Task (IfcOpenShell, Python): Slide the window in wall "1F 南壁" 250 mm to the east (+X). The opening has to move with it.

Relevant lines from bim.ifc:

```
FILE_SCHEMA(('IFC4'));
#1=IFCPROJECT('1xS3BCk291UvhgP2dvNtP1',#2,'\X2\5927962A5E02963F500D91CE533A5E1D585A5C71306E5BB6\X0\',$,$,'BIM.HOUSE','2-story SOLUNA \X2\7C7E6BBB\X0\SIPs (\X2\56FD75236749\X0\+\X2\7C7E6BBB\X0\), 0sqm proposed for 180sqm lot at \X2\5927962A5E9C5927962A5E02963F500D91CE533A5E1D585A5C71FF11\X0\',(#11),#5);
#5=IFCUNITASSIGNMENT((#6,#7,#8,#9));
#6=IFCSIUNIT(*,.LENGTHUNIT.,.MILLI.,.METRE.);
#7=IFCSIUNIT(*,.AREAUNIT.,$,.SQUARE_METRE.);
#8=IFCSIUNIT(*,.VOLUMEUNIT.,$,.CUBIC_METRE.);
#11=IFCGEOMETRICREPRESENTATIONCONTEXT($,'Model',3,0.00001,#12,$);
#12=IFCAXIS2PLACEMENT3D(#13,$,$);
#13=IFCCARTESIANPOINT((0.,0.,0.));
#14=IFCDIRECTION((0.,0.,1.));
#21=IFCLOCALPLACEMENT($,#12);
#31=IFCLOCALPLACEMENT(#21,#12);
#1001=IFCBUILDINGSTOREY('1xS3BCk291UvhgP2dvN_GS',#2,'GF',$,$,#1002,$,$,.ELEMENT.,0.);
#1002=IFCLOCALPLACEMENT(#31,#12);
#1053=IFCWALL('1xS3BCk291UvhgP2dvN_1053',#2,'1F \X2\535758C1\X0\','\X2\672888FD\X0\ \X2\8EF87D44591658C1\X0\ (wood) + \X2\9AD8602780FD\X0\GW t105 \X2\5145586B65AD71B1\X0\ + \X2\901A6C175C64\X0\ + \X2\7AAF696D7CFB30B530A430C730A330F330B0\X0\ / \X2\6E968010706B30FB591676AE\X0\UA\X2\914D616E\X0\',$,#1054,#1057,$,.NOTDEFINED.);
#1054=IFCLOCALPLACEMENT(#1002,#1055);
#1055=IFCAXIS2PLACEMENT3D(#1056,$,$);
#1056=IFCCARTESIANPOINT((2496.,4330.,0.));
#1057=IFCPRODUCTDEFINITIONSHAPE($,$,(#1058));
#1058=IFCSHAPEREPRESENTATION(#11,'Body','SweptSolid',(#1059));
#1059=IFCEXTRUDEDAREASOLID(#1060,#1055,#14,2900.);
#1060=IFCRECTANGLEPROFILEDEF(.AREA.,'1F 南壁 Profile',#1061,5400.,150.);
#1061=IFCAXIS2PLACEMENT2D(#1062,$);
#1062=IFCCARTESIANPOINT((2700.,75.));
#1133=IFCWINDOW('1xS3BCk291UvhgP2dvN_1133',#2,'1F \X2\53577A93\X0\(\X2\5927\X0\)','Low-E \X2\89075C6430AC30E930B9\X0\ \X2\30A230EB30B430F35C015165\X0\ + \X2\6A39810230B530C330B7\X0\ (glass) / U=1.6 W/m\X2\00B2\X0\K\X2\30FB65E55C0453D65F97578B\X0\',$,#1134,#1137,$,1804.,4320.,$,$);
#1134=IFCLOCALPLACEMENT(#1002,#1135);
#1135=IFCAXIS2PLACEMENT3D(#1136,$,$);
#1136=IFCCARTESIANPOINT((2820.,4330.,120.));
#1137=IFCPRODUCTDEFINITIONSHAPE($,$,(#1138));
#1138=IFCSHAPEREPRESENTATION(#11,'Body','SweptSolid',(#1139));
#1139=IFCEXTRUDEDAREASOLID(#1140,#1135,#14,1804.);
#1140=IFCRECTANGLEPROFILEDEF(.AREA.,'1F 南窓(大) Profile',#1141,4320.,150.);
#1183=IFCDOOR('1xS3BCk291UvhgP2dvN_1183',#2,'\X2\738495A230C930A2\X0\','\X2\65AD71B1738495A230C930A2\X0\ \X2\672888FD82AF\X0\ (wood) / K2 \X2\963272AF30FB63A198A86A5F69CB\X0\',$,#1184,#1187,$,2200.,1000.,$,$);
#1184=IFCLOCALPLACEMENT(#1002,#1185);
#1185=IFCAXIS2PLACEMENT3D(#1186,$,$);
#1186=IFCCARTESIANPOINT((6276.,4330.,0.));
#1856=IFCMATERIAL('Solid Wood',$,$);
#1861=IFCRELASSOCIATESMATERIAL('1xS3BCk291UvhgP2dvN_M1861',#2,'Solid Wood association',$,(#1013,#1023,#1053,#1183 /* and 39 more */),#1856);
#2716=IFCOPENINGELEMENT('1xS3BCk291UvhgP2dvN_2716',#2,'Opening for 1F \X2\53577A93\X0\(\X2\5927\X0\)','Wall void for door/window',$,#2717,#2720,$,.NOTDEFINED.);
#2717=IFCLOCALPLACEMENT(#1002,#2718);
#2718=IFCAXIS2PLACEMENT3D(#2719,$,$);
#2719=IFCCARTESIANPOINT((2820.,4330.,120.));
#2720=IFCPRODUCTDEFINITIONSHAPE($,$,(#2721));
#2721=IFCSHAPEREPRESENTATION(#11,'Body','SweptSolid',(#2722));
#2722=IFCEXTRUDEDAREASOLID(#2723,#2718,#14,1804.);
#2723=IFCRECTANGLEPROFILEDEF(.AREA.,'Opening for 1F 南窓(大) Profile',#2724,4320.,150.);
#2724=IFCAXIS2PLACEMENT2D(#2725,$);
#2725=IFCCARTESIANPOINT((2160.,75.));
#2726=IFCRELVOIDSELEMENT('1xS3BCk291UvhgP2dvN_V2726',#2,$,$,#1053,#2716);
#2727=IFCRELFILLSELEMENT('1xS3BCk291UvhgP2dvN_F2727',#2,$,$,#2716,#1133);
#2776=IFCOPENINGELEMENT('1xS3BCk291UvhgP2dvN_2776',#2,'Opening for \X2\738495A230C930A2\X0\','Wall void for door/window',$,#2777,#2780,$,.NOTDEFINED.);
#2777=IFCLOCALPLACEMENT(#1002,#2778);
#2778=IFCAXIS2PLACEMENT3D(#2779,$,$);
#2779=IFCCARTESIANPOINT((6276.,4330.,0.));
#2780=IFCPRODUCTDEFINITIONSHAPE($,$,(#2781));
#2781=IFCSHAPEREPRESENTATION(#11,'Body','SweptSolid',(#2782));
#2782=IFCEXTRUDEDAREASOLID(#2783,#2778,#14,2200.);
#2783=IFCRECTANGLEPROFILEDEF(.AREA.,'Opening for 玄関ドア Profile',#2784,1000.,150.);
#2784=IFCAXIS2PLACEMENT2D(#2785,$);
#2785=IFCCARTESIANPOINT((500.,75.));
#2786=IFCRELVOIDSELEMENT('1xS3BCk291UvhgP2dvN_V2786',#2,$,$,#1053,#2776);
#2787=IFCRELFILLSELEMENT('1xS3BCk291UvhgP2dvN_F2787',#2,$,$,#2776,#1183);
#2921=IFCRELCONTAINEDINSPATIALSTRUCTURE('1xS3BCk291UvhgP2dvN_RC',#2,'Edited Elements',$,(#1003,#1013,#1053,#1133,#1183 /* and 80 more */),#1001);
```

```python
import ifcopenshell
import ifcopenshell.api.geometry
import ifcopenshell.util.placement
import ifcopenshell.util.unit

model = ifcopenshell.open("bim.ifc")
unit_scale = ifcopenshell.util.unit.calculate_unit_scale(model)

window = model.by_guid("1xS3BCk291UvhgP2dvN_1133")
opening = window.FillsVoids[0].RelatingOpeningElement
wall = opening.VoidsElements[0].RelatingBuildingElement

wall_matrix = ifcopenshell.util.placement.get_local_placement(wall.ObjectPlacement)
shift = wall_matrix[:3, 0] * 0.25 / unit_scale
before = ifcopenshell.util.placement.get_local_placement(window.ObjectPlacement)[:3, 3].copy()

# The window is not placed relative to its opening, so move both.
for product in (opening, window):
    matrix = ifcopenshell.util.placement.get_local_placement(product.ObjectPlacement)
    matrix[:3, 3] += shift
    ifcopenshell.api.geometry.edit_object_placement(model, product=product, matrix=matrix, is_si=False)

after = ifcopenshell.util.placement.get_local_placement(window.ObjectPlacement)[:3, 3]
print("window moved by", (after - before).round(3) + 0.0)

model.write("bim-out.ifc")
```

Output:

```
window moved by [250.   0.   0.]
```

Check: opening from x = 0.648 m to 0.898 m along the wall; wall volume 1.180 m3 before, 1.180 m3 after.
